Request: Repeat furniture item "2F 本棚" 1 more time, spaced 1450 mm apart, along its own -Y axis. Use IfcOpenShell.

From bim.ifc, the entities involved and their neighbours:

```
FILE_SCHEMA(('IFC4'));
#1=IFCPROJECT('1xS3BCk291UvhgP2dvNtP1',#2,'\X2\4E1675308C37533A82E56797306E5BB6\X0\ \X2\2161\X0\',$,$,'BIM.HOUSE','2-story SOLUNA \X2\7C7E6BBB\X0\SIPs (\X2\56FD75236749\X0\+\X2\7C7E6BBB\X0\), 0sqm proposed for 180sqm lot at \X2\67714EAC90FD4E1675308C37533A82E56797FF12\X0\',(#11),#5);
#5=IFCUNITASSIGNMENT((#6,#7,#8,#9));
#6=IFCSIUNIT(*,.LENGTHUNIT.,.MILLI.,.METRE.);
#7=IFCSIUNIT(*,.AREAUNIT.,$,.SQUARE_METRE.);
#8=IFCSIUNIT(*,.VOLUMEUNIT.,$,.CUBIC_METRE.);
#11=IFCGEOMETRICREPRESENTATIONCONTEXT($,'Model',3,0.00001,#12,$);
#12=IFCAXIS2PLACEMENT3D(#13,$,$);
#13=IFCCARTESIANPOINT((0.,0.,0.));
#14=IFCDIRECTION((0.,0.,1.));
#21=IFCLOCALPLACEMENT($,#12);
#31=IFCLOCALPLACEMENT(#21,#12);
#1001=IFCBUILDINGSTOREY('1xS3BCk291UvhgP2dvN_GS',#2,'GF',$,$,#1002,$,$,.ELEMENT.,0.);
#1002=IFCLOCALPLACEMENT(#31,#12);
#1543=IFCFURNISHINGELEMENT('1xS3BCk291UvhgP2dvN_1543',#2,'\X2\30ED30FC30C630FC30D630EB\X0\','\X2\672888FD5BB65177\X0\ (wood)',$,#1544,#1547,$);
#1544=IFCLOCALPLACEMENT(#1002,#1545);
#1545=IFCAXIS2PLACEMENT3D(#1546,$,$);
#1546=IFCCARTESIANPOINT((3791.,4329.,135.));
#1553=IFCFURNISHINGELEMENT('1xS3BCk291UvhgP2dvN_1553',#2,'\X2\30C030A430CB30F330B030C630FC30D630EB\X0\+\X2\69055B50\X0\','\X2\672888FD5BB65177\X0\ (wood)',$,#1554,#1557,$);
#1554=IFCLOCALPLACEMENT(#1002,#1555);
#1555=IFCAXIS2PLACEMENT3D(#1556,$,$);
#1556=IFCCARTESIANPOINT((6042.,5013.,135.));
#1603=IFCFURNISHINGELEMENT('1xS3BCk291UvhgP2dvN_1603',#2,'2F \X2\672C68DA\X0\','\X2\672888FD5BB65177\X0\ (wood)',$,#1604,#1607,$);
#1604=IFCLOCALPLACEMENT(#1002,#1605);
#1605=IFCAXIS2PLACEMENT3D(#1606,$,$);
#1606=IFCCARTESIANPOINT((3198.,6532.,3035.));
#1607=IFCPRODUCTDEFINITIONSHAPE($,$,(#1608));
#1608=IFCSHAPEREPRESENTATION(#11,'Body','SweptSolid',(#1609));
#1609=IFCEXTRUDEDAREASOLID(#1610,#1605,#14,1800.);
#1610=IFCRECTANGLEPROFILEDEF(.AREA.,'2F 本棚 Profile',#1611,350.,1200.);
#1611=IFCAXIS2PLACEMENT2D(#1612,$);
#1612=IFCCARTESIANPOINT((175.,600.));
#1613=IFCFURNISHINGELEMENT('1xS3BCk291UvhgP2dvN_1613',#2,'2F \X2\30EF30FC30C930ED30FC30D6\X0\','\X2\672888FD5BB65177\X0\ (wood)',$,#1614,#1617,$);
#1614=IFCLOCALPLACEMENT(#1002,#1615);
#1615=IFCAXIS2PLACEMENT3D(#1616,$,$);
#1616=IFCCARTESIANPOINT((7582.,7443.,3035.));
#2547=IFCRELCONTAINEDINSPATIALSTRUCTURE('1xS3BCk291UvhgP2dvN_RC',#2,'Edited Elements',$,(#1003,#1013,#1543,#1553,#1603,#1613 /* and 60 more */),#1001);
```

```python
import ifcopenshell
import ifcopenshell.api.geometry
import ifcopenshell.api.root
import ifcopenshell.util.element
import ifcopenshell.util.placement

model = ifcopenshell.open("bim.ifc")


def reuse_history(source, copy):
    """copy_class also copies each property set's owner history, people and application; keep the originals."""
    for rel in copy.IsDefinedBy:
        if rel.is_a("IfcRelDefinesByProperties") and (history := rel.RelatingPropertyDefinition.OwnerHistory):
            rel.RelatingPropertyDefinition.OwnerHistory = source.OwnerHistory
            ifcopenshell.util.element.remove_deep2(model, history)


source = model.by_id(1603)
base = ifcopenshell.util.placement.get_local_placement(source.ObjectPlacement)
step = -base[:3, 1] * 1450.0

for i in range(1, 2):
    copy = ifcopenshell.api.root.copy_class(model, product=source)
    copy.Representation = ifcopenshell.util.element.copy_deep(
        model, source.Representation, exclude=["IfcGeometricRepresentationContext", "IfcRepresentationMap"]
    )
    reuse_history(source, copy)
    matrix = base.copy()
    matrix[:3, 3] += i * step
    print("added at", matrix[:3, 3].round(3) + 0.0)
    ifcopenshell.api.geometry.edit_object_placement(model, product=copy, matrix=matrix, is_si=False)

model.write("bim_edited.ifc")
```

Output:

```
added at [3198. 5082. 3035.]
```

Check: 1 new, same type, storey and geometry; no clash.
